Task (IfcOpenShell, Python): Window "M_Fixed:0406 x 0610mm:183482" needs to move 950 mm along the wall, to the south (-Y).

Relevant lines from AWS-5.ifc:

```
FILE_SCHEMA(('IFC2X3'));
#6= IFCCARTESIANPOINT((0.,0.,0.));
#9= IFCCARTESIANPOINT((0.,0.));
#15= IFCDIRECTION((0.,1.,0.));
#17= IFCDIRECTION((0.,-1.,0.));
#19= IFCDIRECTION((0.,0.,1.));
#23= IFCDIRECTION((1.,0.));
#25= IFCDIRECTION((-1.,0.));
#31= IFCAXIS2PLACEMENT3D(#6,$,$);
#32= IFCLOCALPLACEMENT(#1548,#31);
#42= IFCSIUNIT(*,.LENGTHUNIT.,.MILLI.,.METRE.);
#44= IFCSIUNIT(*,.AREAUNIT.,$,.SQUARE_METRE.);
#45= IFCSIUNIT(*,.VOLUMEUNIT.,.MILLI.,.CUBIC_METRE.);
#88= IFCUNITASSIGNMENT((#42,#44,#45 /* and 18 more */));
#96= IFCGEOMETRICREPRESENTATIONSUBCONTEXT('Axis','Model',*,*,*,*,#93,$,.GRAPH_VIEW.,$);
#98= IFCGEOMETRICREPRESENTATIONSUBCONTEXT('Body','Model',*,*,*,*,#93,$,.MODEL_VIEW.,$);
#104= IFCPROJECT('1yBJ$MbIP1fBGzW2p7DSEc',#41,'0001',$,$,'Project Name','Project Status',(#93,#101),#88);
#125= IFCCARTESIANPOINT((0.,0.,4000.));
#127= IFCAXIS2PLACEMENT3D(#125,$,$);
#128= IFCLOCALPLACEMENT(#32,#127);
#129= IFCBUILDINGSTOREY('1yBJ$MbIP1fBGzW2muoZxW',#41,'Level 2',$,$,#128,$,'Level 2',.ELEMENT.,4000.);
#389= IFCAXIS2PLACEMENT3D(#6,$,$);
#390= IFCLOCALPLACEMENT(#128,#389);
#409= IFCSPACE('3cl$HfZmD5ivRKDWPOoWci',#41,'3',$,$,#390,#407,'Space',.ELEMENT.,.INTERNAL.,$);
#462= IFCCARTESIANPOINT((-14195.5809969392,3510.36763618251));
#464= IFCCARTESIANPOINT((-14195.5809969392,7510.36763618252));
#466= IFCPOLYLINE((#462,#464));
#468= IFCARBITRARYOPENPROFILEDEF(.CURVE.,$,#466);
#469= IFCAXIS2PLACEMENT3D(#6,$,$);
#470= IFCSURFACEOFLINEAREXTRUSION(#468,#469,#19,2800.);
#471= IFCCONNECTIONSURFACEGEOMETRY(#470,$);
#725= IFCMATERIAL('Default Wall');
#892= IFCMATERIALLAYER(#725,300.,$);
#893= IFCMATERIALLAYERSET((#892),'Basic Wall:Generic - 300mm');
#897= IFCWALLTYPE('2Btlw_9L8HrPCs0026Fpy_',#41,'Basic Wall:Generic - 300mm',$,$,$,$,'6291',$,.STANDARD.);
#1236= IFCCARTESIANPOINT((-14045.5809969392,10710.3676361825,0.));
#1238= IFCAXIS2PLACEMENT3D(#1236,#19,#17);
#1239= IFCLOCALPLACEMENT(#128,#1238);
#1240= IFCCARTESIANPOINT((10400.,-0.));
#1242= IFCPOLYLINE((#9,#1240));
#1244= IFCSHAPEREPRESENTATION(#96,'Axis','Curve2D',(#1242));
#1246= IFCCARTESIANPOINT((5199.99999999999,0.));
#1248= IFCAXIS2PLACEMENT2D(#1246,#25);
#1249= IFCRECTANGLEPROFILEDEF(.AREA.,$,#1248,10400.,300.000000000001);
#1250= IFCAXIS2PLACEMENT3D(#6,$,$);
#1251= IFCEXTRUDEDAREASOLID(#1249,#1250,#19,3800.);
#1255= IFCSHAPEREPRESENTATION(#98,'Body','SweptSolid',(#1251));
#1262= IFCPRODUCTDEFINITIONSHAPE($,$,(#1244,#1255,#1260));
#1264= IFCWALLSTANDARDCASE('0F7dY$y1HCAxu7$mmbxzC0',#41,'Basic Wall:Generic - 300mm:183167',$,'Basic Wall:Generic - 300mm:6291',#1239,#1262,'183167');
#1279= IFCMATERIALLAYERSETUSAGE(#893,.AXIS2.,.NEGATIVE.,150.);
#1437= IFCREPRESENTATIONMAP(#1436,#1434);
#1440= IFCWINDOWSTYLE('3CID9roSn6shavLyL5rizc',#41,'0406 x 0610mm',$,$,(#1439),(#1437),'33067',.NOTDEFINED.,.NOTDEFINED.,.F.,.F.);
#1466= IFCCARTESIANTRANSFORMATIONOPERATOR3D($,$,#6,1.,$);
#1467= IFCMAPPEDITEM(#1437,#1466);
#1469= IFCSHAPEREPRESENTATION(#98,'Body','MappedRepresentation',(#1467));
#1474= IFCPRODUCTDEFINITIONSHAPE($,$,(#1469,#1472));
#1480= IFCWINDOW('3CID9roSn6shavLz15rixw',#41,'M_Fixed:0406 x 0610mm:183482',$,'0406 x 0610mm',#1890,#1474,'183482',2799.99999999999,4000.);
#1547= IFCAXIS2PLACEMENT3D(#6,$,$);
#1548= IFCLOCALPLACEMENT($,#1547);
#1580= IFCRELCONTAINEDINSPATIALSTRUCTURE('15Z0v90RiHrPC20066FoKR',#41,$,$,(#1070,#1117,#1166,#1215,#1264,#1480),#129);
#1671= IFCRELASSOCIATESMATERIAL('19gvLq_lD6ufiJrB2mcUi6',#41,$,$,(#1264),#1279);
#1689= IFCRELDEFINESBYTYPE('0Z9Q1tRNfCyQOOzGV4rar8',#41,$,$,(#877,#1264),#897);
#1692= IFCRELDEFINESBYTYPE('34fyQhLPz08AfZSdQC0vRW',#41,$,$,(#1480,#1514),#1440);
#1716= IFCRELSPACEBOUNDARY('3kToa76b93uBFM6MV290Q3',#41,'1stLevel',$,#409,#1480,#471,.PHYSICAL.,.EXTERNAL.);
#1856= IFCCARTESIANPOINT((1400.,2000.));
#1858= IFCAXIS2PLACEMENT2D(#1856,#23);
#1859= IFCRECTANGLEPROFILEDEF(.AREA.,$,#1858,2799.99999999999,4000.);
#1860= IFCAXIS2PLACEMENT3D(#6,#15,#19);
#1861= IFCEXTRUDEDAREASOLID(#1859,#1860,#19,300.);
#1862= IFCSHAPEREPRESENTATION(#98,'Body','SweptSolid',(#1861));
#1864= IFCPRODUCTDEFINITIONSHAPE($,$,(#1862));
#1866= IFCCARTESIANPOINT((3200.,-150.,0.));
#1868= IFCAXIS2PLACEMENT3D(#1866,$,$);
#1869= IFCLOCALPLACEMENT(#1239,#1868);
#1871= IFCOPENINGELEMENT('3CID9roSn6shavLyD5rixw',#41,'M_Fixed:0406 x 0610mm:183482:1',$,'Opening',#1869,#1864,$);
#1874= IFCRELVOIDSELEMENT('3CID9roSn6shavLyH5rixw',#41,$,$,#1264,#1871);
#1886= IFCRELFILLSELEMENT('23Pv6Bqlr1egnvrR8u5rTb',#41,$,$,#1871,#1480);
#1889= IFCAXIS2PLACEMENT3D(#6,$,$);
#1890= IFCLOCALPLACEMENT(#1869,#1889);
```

```python
import numpy as np
import ifcopenshell
import ifcopenshell.api.geometry
import ifcopenshell.util.placement

model = ifcopenshell.open("AWS-5.ifc")

window = model.by_id(1480)
opening = window.FillsVoids[0].RelatingOpeningElement
wall = opening.VoidsElements[0].RelatingBuildingElement

wall_matrix = ifcopenshell.util.placement.get_local_placement(wall.ObjectPlacement)
shift = wall_matrix[:3, 0] * 950.0
before = ifcopenshell.util.placement.get_local_placement(window.ObjectPlacement)[:3, 3].copy()

# The window is placed relative to its opening, so it follows when the opening moves.
matrix = ifcopenshell.util.placement.get_local_placement(opening.ObjectPlacement)
matrix[:3, 3] += shift
ifcopenshell.api.geometry.edit_object_placement(
    model, product=opening, matrix=matrix, is_si=False, should_transform_children=True
)

# Space boundary surfaces are stored in each space's coordinates; move them too.
for rel in window.ProvidesBoundaries:
    if not rel.ConnectionGeometry:
        continue
    surface = rel.ConnectionGeometry.SurfaceOnRelatingElement
    space_matrix = ifcopenshell.util.placement.get_local_placement(rel.RelatingSpace.ObjectPlacement)
    point = np.array(surface.Position.Location.Coordinates) + space_matrix[:3, :3].T @ shift
    surface.Position = model.createIfcAxis2Placement3D(
        model.createIfcCartesianPoint(point.tolist()), surface.Position.Axis, surface.Position.RefDirection
    )

after = ifcopenshell.util.placement.get_local_placement(window.ObjectPlacement)[:3, 3]
print("window moved by", (after - before).round(3) + 0.0)

model.write("AWS-5_rev.ifc")
```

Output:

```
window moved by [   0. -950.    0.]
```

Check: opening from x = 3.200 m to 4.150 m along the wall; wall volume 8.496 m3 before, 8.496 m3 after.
